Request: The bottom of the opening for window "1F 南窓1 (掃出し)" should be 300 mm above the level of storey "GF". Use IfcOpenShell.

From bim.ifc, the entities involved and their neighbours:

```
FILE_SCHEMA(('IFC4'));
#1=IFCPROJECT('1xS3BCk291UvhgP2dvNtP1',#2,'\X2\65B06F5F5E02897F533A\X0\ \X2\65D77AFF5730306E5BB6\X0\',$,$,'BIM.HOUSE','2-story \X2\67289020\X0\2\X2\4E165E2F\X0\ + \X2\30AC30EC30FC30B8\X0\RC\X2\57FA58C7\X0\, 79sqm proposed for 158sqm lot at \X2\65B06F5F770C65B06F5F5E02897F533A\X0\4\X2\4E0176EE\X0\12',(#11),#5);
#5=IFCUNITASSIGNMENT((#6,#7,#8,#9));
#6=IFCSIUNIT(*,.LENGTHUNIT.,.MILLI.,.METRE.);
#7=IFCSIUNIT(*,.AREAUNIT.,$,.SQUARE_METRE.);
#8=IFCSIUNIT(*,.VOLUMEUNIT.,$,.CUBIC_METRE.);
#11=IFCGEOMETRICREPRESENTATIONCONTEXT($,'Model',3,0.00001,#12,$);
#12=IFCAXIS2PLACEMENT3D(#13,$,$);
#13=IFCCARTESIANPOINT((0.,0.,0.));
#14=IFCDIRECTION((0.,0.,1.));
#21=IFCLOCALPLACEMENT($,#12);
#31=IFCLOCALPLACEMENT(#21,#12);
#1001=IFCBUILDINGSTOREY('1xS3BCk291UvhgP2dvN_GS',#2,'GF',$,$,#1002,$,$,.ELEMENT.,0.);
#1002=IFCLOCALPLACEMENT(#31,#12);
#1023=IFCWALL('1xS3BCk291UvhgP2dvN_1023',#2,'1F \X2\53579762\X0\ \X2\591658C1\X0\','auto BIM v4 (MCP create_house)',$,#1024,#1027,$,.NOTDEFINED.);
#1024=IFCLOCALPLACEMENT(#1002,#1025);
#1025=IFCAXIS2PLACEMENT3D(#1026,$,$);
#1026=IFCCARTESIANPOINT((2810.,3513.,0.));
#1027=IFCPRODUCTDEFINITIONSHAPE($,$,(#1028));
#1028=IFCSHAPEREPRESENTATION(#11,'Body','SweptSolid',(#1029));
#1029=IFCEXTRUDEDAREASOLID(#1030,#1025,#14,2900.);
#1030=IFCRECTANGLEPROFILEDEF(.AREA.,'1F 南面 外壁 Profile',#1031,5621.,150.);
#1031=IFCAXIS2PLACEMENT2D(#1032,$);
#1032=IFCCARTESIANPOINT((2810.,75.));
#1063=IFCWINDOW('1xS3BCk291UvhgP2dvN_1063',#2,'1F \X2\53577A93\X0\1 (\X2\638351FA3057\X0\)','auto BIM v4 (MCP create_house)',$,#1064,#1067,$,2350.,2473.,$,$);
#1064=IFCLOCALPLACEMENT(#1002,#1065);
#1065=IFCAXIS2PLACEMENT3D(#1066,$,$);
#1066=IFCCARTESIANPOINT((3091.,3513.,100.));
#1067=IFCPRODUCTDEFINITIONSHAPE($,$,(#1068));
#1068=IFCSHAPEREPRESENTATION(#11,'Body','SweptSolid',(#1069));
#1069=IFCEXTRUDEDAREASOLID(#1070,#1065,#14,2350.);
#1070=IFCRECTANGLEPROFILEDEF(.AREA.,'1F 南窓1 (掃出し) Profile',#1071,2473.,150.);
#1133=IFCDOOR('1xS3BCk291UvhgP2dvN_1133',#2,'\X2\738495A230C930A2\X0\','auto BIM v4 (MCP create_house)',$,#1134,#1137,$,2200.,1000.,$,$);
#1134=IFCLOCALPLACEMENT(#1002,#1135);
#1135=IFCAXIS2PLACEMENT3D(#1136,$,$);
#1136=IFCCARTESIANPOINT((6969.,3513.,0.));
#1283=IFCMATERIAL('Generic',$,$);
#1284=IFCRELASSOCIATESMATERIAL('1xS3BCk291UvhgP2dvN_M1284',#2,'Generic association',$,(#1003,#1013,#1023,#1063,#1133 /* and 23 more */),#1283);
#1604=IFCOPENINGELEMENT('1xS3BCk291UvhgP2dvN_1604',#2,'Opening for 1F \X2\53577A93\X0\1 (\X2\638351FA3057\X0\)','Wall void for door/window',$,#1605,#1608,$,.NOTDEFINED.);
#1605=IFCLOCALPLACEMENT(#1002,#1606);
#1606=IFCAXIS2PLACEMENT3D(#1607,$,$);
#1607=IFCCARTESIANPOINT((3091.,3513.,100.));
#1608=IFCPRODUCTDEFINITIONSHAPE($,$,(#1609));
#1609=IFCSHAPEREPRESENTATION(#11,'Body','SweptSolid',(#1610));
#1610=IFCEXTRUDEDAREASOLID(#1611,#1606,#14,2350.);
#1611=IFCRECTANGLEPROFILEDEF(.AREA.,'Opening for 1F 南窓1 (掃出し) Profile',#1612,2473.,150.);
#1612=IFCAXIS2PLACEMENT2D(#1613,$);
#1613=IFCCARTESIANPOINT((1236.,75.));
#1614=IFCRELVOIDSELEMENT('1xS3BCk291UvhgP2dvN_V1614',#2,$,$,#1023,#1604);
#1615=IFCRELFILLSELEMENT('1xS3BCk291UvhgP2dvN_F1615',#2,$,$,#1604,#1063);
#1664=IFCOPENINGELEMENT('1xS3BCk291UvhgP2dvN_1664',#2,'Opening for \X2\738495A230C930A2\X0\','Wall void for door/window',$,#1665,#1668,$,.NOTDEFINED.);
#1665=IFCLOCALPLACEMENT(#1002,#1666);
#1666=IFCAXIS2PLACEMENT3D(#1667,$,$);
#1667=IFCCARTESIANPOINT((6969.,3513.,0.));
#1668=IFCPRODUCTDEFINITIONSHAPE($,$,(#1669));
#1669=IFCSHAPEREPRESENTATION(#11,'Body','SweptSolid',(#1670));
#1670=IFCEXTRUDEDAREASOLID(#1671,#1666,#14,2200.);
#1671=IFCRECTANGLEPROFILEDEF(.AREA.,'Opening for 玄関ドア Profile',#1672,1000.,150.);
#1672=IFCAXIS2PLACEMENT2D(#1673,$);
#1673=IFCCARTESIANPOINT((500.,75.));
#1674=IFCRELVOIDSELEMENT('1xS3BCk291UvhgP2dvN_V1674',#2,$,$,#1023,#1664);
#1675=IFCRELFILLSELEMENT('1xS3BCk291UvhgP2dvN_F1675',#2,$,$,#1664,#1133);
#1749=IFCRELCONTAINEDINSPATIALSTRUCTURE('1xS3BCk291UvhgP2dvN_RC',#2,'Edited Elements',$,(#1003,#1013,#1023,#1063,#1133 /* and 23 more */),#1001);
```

```python
import numpy as np
import ifcopenshell
import ifcopenshell.api.geometry
import ifcopenshell.geom
import ifcopenshell.util.element
import ifcopenshell.util.placement
import ifcopenshell.util.shape
import ifcopenshell.util.unit

model = ifcopenshell.open("bim.ifc")
unit_scale = ifcopenshell.util.unit.calculate_unit_scale(model)

window = model.by_id(1063)
opening = window.FillsVoids[0].RelatingOpeningElement
storey = ifcopenshell.util.element.get_container(window, ifc_class="IfcBuildingStorey")
level = ifcopenshell.util.placement.get_local_placement(storey.ObjectPlacement)[2, 3]

# The opening's origin need not be at the sill, so measure its lowest point.
shape = ifcopenshell.geom.create_shape(ifcopenshell.geom.settings(), opening)
bottom = ifcopenshell.util.shape.get_shape_bottom_elevation(shape, shape.geometry) / unit_scale
dz = level + 300.0 - bottom

shift = np.array([0.0, 0.0, dz])
# The window is not placed relative to its opening, so move both.
for product in (opening, window):
    matrix = ifcopenshell.util.placement.get_local_placement(product.ObjectPlacement)
    matrix[:3, 3] += shift
    ifcopenshell.api.geometry.edit_object_placement(model, product=product, matrix=matrix, is_si=False)

print(f"moved by {dz * unit_scale:+.3f} m")

model.write("bim_rev.ifc")
```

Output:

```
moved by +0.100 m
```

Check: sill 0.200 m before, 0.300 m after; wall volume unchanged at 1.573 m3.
